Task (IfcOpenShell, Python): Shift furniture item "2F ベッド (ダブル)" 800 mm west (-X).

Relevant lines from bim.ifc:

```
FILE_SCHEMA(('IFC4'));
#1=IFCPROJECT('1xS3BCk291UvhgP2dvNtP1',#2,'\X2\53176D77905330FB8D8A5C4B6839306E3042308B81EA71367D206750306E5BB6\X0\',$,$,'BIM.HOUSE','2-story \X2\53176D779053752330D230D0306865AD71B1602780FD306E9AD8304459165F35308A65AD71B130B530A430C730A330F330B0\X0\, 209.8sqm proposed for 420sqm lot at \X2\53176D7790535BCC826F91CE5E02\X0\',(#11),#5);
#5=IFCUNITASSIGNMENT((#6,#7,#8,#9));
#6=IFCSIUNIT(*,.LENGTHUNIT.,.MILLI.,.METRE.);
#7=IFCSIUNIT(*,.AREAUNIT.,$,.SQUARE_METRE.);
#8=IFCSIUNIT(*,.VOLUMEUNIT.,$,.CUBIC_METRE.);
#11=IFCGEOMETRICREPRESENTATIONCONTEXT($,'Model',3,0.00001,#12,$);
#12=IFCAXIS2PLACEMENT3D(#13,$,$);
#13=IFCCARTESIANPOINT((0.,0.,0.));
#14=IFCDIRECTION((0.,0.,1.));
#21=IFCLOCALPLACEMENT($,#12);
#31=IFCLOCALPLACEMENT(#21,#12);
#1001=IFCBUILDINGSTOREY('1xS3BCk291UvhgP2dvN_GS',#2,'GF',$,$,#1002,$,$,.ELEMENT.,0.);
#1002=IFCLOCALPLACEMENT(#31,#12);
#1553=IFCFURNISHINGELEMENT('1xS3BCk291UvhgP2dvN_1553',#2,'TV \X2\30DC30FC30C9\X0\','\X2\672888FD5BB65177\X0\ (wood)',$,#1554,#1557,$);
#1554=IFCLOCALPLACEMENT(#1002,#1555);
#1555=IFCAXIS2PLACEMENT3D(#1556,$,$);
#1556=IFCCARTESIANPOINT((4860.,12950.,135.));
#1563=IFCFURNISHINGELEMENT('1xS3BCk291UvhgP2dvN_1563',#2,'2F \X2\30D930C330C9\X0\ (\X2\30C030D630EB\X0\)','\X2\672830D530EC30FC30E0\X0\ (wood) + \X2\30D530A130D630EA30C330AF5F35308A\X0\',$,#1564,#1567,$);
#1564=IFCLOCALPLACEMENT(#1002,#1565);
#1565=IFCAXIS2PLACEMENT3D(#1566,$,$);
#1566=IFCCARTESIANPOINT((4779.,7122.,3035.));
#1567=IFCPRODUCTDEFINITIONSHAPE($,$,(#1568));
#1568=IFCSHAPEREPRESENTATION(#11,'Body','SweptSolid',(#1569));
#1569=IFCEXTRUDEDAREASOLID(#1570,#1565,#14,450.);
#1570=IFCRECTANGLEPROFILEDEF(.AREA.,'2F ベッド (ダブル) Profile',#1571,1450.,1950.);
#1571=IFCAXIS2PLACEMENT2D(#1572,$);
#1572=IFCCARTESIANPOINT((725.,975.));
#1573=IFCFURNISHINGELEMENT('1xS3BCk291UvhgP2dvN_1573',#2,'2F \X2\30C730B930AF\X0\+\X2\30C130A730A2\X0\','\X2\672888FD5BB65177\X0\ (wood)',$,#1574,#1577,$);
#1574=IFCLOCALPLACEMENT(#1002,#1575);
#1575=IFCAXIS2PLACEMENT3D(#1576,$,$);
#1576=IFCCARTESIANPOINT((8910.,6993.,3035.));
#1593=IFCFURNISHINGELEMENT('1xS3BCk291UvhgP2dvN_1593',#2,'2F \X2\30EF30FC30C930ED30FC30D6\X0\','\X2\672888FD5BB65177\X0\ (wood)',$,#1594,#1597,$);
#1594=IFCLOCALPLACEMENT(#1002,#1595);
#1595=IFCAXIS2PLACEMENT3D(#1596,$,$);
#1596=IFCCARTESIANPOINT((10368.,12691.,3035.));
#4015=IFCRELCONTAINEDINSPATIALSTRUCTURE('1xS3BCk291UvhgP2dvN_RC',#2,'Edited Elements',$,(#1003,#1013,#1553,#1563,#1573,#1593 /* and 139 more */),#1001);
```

```python
import ifcopenshell
import ifcopenshell.api.geometry
import ifcopenshell.util.placement
import ifcopenshell.util.unit

model = ifcopenshell.open("bim.ifc")
unit_scale = ifcopenshell.util.unit.calculate_unit_scale(model)

item = model.by_guid("1xS3BCk291UvhgP2dvN_1563")
matrix = ifcopenshell.util.placement.get_local_placement(item.ObjectPlacement)
matrix[0, 3] -= 0.8 / unit_scale
ifcopenshell.api.geometry.edit_object_placement(model, product=item, matrix=matrix, is_si=False)

print(ifcopenshell.util.placement.get_local_placement(item.ObjectPlacement).round(3) + 0.0)

model.write("bim_updated.ifc")
```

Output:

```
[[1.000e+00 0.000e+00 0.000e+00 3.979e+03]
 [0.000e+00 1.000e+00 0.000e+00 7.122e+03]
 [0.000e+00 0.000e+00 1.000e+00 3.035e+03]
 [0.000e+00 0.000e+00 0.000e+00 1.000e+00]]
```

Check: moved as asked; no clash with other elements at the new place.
